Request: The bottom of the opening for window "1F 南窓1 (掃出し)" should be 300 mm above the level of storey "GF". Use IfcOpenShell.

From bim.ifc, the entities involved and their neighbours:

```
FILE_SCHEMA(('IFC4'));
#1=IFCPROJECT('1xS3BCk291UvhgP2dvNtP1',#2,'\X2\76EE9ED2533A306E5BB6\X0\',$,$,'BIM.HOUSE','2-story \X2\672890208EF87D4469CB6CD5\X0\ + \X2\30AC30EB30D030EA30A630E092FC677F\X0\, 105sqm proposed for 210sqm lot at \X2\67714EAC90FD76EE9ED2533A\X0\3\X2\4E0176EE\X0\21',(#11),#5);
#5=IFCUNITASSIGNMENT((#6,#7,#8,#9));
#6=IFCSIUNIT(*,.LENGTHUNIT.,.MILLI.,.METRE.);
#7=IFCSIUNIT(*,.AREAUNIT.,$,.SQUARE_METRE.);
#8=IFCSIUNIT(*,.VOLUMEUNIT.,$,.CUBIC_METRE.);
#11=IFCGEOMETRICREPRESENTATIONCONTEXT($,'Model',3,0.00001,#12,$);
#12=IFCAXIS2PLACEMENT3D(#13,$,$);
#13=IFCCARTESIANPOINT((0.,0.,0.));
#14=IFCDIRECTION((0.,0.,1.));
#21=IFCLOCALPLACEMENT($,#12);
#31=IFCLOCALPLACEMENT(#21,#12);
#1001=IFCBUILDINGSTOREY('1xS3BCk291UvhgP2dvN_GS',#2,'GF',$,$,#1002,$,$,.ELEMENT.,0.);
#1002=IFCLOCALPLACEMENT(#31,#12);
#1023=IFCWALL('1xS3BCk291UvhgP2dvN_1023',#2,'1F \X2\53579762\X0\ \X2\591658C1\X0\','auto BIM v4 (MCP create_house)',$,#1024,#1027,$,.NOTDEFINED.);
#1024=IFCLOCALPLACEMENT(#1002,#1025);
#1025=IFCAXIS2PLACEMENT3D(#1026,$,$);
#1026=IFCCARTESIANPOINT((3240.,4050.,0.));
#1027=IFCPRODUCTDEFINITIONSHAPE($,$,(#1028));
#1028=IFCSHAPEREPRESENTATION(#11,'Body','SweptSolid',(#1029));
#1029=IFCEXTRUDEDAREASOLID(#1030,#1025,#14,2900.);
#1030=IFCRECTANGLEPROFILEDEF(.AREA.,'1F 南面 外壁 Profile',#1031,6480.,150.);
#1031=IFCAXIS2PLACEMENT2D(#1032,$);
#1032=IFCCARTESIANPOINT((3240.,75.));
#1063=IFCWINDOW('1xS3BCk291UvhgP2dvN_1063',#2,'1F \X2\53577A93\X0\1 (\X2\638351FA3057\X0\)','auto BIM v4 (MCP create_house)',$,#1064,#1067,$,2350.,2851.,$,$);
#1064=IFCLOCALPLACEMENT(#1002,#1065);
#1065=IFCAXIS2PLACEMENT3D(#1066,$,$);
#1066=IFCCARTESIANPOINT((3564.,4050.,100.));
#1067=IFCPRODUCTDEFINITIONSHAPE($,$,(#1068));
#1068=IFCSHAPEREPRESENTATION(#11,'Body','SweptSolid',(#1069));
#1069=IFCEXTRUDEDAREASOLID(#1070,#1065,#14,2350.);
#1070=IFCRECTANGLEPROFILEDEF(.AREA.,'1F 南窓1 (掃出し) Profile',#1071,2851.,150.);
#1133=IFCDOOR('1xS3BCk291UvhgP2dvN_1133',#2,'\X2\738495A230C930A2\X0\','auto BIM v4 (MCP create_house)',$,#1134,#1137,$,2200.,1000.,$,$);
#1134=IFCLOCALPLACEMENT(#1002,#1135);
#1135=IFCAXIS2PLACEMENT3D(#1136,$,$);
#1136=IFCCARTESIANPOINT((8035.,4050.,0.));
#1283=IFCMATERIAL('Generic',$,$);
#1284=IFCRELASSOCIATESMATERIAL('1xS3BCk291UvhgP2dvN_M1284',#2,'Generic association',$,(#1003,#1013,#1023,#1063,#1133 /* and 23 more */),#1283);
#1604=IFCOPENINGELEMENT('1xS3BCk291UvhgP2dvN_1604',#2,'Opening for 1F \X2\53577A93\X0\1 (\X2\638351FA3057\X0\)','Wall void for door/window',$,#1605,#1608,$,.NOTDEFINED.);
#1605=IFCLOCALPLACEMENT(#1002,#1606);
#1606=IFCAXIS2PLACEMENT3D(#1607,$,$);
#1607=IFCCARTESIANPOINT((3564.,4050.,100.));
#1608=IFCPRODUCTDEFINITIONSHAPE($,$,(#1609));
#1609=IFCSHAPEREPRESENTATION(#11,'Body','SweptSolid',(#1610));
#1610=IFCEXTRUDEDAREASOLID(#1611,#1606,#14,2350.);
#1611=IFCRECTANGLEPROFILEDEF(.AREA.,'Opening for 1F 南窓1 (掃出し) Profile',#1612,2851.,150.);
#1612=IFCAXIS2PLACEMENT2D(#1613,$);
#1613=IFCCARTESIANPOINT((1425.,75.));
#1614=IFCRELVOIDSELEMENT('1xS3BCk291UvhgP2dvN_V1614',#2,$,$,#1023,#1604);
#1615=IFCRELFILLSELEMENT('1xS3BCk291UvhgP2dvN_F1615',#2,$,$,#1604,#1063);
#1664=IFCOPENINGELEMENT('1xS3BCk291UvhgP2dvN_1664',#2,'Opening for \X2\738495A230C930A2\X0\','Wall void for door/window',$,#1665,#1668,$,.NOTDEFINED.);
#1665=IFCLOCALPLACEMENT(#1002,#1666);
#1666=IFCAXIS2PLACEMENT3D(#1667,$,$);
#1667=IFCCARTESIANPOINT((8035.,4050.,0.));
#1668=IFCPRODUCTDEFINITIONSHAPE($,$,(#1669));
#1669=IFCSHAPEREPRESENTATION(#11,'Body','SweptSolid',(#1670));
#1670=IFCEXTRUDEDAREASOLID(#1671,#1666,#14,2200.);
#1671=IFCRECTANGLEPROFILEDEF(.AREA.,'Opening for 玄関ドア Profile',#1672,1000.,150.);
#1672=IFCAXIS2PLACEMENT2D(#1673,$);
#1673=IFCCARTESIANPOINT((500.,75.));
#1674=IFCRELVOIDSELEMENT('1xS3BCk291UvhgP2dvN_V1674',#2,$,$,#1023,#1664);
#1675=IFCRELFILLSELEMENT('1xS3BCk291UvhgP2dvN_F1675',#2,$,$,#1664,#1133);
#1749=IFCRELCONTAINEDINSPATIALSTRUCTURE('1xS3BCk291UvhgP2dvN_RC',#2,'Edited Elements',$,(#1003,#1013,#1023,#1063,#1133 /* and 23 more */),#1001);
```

```python
import numpy as np
import ifcopenshell
import ifcopenshell.api.geometry
import ifcopenshell.geom
import ifcopenshell.util.element
import ifcopenshell.util.placement
import ifcopenshell.util.shape
import ifcopenshell.util.unit

model = ifcopenshell.open("bim.ifc")
unit_scale = ifcopenshell.util.unit.calculate_unit_scale(model)

window = model.by_guid("1xS3BCk291UvhgP2dvN_1063")
opening = window.FillsVoids[0].RelatingOpeningElement
storey = ifcopenshell.util.element.get_container(window, ifc_class="IfcBuildingStorey")
level = ifcopenshell.util.placement.get_local_placement(storey.ObjectPlacement)[2, 3]

# The opening's origin need not be at the sill, so measure its lowest point.
shape = ifcopenshell.geom.create_shape(ifcopenshell.geom.settings(), opening)
bottom = ifcopenshell.util.shape.get_shape_bottom_elevation(shape, shape.geometry) / unit_scale
dz = level + 300.0 - bottom

shift = np.array([0.0, 0.0, dz])
# The window is not placed relative to its opening, so move both.
for product in (opening, window):
    matrix = ifcopenshell.util.placement.get_local_placement(product.ObjectPlacement)
    matrix[:3, 3] += shift
    ifcopenshell.api.geometry.edit_object_placement(model, product=product, matrix=matrix, is_si=False)

print(f"moved by {dz * unit_scale:+.3f} m")

model.write("bim_v2.ifc")
```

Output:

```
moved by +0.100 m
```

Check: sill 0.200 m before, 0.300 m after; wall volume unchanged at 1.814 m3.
